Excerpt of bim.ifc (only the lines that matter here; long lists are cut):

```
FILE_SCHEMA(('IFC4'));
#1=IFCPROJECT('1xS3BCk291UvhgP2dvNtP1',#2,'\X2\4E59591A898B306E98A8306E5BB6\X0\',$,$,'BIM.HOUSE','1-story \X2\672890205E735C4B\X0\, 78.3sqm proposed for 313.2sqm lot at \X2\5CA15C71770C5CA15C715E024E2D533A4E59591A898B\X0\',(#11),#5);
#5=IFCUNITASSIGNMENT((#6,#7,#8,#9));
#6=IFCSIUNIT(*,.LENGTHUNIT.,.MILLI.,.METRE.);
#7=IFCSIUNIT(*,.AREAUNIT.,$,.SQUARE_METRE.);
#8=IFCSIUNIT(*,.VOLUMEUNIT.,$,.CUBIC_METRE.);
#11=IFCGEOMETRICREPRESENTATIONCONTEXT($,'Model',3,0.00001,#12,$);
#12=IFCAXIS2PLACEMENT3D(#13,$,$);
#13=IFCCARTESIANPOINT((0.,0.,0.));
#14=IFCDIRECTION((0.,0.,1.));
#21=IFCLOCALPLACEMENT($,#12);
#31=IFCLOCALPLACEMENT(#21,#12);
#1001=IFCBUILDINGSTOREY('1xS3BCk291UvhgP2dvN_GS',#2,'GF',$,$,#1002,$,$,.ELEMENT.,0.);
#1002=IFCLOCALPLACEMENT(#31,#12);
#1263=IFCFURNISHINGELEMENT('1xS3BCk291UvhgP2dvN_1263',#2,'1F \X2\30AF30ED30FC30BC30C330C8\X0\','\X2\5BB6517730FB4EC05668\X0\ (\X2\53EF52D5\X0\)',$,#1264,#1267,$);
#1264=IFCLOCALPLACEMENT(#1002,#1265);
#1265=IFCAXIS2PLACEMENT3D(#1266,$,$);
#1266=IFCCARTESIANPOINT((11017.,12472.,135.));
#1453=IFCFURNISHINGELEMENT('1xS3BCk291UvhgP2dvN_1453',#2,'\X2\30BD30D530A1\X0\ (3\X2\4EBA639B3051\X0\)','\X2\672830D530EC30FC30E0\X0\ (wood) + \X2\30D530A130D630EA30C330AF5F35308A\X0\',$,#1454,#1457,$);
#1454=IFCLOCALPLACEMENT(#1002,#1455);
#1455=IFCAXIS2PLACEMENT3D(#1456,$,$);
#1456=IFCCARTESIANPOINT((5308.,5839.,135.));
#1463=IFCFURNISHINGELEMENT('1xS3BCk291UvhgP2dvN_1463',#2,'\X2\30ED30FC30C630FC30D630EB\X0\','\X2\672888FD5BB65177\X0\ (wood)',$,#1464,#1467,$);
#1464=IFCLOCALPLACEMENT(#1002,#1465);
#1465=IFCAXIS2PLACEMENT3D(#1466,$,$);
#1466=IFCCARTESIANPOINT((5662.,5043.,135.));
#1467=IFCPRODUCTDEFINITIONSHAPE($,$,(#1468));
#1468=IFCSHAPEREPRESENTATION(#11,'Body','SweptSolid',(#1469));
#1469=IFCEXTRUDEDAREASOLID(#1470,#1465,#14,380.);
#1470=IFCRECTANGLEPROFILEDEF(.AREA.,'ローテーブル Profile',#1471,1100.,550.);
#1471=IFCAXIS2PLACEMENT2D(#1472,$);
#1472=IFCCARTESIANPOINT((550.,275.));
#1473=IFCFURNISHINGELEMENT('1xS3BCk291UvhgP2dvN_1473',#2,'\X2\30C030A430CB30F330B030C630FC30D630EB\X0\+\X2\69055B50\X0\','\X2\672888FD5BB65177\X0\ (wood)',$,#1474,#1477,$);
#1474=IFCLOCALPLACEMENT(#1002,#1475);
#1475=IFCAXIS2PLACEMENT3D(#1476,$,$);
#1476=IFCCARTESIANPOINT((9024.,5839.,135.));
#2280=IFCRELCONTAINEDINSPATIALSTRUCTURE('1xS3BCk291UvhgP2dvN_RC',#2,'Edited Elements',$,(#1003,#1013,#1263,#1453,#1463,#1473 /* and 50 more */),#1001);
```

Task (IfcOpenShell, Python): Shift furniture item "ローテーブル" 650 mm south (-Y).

```python
import ifcopenshell
import ifcopenshell.api.geometry
import ifcopenshell.util.placement

model = ifcopenshell.open("bim.ifc")

item = model.by_guid("1xS3BCk291UvhgP2dvN_1463")
matrix = ifcopenshell.util.placement.get_local_placement(item.ObjectPlacement)
matrix[1, 3] -= 650.0
ifcopenshell.api.geometry.edit_object_placement(model, product=item, matrix=matrix, is_si=False)

print(ifcopenshell.util.placement.get_local_placement(item.ObjectPlacement).round(3) + 0.0)

model.write("bim_edited.ifc")
```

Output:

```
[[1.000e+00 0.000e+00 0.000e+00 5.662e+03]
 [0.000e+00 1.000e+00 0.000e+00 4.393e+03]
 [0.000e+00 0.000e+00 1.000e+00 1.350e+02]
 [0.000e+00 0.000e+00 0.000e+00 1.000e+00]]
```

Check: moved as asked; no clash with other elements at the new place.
